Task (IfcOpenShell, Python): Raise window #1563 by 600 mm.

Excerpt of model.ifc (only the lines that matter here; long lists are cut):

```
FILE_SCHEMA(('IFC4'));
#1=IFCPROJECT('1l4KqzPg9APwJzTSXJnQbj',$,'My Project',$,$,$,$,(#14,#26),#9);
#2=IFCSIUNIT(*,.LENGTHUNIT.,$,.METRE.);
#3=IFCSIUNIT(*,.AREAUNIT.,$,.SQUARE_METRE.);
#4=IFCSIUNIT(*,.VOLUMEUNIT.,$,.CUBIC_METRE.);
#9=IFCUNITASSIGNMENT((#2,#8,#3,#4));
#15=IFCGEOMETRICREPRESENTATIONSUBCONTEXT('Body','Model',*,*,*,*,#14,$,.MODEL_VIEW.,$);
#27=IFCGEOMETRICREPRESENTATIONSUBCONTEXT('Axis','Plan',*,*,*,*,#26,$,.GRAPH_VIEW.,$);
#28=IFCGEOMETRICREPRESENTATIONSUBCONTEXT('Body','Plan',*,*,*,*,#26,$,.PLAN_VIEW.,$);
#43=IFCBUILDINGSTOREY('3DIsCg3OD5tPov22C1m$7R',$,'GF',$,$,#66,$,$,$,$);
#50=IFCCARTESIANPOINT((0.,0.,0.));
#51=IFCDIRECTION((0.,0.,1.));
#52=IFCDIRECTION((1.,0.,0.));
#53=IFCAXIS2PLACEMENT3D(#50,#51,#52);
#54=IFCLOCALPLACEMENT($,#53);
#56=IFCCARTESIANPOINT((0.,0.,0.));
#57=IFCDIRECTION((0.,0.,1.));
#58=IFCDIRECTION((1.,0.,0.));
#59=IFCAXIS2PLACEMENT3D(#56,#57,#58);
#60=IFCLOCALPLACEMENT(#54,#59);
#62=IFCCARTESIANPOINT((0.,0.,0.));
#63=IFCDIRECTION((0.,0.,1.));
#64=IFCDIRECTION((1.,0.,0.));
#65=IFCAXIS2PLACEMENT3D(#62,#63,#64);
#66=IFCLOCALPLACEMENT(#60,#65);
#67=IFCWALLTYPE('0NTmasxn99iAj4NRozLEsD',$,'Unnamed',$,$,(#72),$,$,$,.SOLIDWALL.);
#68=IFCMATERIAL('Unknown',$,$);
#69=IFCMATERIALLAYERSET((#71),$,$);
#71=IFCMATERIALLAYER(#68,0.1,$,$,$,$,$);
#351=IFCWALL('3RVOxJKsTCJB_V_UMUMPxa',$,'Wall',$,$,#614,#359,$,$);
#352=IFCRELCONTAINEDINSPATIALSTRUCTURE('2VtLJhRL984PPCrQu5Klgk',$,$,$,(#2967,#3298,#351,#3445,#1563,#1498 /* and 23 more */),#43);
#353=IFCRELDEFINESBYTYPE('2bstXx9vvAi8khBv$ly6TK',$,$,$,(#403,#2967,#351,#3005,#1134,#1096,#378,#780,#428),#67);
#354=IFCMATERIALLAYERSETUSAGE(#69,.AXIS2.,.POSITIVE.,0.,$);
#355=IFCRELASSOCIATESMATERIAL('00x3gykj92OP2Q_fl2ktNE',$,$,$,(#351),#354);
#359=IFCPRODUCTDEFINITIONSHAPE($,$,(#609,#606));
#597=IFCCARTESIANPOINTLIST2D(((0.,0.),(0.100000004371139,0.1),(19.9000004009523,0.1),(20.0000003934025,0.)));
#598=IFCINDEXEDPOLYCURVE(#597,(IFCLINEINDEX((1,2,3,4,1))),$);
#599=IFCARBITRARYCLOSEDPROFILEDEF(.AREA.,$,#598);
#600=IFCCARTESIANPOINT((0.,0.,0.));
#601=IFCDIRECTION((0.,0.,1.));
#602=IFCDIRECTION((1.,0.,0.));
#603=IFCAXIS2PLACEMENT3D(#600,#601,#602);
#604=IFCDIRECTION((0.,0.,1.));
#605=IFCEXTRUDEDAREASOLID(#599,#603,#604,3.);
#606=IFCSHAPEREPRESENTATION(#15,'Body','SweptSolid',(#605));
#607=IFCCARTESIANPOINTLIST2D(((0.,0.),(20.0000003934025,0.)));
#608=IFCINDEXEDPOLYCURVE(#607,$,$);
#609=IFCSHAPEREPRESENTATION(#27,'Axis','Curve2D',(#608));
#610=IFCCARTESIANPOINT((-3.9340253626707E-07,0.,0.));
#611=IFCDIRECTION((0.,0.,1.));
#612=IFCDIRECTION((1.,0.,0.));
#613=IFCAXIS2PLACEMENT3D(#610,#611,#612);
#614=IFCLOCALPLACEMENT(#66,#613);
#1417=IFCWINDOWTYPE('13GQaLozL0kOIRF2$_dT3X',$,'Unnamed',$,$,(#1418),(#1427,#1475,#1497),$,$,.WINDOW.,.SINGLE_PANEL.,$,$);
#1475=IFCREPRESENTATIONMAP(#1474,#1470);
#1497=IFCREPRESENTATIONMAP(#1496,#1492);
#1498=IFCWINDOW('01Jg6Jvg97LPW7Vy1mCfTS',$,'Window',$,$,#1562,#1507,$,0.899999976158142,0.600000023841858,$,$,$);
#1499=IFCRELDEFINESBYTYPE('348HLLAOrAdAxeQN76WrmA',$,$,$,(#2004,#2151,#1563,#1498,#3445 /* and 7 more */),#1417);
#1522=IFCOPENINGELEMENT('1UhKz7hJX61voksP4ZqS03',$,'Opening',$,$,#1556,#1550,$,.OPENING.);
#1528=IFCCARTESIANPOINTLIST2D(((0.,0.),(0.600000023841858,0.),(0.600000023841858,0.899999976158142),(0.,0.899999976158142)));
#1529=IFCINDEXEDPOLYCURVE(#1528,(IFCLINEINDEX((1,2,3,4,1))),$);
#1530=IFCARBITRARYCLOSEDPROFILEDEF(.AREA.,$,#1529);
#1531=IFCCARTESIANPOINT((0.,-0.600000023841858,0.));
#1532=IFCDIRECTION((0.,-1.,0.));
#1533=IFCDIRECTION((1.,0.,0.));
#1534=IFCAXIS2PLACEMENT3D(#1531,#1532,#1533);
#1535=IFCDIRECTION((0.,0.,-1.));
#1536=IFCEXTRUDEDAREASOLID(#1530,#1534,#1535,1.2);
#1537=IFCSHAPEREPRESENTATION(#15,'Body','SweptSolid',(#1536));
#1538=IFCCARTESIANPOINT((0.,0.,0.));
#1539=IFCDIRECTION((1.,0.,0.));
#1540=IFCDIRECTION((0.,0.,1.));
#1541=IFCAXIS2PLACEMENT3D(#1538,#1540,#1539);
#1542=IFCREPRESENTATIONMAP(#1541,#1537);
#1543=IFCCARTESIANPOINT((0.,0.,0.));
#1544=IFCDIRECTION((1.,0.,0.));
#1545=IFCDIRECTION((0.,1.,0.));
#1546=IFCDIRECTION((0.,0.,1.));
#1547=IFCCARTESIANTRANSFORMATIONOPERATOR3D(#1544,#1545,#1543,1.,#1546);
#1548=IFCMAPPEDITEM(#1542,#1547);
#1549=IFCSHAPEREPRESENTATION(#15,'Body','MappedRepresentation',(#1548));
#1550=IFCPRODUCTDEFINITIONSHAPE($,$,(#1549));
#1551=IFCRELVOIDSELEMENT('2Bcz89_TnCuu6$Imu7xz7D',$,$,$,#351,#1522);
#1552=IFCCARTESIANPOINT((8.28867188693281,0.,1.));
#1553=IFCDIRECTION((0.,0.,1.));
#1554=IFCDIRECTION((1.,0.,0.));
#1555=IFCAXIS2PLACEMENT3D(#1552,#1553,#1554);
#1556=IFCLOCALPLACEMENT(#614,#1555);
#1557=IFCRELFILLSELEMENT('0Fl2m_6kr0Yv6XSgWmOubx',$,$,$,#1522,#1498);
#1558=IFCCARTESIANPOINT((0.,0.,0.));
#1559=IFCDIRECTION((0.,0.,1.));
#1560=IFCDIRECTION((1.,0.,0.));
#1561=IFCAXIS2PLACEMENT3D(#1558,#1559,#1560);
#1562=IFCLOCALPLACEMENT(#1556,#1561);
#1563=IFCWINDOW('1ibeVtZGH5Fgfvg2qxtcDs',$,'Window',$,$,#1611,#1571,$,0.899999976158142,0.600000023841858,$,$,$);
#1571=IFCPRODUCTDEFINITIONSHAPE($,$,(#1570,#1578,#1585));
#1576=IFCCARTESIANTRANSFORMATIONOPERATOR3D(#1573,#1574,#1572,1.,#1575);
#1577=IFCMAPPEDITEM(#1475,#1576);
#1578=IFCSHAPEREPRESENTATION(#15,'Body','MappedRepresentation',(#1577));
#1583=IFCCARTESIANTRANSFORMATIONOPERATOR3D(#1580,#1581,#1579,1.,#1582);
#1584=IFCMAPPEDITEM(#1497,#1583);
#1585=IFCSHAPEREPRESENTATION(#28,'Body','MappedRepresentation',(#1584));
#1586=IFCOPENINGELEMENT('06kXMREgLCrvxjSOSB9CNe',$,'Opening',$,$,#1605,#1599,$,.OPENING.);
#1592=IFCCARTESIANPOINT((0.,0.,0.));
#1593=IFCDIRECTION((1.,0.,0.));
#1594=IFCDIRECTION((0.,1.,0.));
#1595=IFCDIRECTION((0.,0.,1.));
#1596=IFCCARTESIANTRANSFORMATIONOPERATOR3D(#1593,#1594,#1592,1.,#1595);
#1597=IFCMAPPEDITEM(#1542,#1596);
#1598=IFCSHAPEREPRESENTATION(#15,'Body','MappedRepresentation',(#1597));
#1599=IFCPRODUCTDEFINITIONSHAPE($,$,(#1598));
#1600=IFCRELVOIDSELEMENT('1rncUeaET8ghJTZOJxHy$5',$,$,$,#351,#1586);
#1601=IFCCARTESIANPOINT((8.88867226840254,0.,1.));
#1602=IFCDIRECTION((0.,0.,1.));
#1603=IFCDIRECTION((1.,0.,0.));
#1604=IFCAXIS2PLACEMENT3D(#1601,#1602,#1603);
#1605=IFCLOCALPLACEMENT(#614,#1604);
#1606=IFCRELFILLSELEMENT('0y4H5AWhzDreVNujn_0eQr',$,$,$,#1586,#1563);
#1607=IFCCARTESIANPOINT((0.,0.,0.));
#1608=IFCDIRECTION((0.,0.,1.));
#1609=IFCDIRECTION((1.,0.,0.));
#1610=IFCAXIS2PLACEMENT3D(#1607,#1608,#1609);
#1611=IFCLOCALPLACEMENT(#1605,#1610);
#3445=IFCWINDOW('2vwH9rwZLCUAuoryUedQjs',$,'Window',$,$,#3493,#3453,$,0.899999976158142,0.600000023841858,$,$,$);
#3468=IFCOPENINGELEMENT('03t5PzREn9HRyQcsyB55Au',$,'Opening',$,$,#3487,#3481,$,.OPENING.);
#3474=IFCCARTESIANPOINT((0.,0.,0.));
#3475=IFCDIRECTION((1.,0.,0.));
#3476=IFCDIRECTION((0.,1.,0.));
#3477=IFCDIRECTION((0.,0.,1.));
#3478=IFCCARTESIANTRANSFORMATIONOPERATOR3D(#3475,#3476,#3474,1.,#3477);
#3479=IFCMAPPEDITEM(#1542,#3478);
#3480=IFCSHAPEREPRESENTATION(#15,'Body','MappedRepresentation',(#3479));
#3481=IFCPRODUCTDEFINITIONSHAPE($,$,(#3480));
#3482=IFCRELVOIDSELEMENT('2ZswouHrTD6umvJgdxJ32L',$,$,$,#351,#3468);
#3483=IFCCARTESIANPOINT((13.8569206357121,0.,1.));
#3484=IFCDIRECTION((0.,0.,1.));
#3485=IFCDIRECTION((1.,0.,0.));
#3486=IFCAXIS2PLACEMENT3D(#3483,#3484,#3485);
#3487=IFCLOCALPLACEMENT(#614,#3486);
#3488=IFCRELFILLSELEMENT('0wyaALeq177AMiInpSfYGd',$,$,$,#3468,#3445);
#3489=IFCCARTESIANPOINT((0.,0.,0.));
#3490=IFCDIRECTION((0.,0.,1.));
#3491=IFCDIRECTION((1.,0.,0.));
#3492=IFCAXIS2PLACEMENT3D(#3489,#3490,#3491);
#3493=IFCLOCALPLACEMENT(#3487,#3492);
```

```python
import numpy as np
import ifcopenshell
import ifcopenshell.api.geometry
import ifcopenshell.util.placement
import ifcopenshell.util.unit

model = ifcopenshell.open("model.ifc")
unit_scale = ifcopenshell.util.unit.calculate_unit_scale(model)

window = model.by_guid("1ibeVtZGH5Fgfvg2qxtcDs")
opening = window.FillsVoids[0].RelatingOpeningElement
dz = 0.6 / unit_scale

shift = np.array([0.0, 0.0, dz])
# The window is placed relative to its opening, so it follows when the opening moves.
matrix = ifcopenshell.util.placement.get_local_placement(opening.ObjectPlacement)
matrix[:3, 3] += shift
ifcopenshell.api.geometry.edit_object_placement(
    model, product=opening, matrix=matrix, is_si=False, should_transform_children=True
)

print(f"moved by {dz * unit_scale:+.3f} m")

model.write("model_edited.ifc")
```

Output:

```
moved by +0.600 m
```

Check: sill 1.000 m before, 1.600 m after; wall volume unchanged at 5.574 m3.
